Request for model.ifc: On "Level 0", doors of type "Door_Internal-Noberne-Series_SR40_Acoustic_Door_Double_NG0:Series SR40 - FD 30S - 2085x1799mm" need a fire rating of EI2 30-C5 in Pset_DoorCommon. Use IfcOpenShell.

First a look at what the model holds.

```python
import ifcopenshell
import ifcopenshell.util.element

model = ifcopenshell.open("model.ifc")
print(model.schema)
storey = next(s for s in model.by_type("IfcBuildingStorey") if s.Name == "Level 0")
doors = [e for e in ifcopenshell.util.element.get_decomposition(storey) if e.is_a("IfcDoor")]
seen = {}
for e in doors:
    element_type = ifcopenshell.util.element.get_type(e)
    key = (element_type.Name if element_type != e and element_type else None, ifcopenshell.util.element.get_pset(e, "Pset_DoorCommon", "FireRating"))
    seen[key] = seen.get(key, 0) + 1
for (name, value), count in sorted(seen.items(), key=str):
    print(count, "x", name, "|", value)
```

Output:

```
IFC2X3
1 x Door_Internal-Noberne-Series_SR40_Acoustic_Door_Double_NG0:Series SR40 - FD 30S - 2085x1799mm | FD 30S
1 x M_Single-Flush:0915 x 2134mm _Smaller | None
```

```python
import ifcopenshell
import ifcopenshell.api.pset
import ifcopenshell.util.element

model = ifcopenshell.open("model.ifc")

storey = next(s for s in model.by_type("IfcBuildingStorey") if s.Name == "Level 0")
doors = [e for e in ifcopenshell.util.element.get_decomposition(storey) if e.is_a("IfcDoor")]

count = 0
for e in doors:
    element_type = ifcopenshell.util.element.get_type(e)
    if element_type in (None, e) or element_type.Name != "Door_Internal-Noberne-Series_SR40_Acoustic_Door_Double_NG0:Series SR40 - FD 30S - 2085x1799mm":
        continue
    # add_pset returns the element's existing set when there is one.
    pset = ifcopenshell.api.pset.add_pset(model, product=e, name="Pset_DoorCommon")
    ifcopenshell.api.pset.edit_pset(model, pset=pset, properties={"FireRating": "EI2 30-C5"})
    count += 1

print(count, "doors updated")

model.write("model_updated.ifc")
```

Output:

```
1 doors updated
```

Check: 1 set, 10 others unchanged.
